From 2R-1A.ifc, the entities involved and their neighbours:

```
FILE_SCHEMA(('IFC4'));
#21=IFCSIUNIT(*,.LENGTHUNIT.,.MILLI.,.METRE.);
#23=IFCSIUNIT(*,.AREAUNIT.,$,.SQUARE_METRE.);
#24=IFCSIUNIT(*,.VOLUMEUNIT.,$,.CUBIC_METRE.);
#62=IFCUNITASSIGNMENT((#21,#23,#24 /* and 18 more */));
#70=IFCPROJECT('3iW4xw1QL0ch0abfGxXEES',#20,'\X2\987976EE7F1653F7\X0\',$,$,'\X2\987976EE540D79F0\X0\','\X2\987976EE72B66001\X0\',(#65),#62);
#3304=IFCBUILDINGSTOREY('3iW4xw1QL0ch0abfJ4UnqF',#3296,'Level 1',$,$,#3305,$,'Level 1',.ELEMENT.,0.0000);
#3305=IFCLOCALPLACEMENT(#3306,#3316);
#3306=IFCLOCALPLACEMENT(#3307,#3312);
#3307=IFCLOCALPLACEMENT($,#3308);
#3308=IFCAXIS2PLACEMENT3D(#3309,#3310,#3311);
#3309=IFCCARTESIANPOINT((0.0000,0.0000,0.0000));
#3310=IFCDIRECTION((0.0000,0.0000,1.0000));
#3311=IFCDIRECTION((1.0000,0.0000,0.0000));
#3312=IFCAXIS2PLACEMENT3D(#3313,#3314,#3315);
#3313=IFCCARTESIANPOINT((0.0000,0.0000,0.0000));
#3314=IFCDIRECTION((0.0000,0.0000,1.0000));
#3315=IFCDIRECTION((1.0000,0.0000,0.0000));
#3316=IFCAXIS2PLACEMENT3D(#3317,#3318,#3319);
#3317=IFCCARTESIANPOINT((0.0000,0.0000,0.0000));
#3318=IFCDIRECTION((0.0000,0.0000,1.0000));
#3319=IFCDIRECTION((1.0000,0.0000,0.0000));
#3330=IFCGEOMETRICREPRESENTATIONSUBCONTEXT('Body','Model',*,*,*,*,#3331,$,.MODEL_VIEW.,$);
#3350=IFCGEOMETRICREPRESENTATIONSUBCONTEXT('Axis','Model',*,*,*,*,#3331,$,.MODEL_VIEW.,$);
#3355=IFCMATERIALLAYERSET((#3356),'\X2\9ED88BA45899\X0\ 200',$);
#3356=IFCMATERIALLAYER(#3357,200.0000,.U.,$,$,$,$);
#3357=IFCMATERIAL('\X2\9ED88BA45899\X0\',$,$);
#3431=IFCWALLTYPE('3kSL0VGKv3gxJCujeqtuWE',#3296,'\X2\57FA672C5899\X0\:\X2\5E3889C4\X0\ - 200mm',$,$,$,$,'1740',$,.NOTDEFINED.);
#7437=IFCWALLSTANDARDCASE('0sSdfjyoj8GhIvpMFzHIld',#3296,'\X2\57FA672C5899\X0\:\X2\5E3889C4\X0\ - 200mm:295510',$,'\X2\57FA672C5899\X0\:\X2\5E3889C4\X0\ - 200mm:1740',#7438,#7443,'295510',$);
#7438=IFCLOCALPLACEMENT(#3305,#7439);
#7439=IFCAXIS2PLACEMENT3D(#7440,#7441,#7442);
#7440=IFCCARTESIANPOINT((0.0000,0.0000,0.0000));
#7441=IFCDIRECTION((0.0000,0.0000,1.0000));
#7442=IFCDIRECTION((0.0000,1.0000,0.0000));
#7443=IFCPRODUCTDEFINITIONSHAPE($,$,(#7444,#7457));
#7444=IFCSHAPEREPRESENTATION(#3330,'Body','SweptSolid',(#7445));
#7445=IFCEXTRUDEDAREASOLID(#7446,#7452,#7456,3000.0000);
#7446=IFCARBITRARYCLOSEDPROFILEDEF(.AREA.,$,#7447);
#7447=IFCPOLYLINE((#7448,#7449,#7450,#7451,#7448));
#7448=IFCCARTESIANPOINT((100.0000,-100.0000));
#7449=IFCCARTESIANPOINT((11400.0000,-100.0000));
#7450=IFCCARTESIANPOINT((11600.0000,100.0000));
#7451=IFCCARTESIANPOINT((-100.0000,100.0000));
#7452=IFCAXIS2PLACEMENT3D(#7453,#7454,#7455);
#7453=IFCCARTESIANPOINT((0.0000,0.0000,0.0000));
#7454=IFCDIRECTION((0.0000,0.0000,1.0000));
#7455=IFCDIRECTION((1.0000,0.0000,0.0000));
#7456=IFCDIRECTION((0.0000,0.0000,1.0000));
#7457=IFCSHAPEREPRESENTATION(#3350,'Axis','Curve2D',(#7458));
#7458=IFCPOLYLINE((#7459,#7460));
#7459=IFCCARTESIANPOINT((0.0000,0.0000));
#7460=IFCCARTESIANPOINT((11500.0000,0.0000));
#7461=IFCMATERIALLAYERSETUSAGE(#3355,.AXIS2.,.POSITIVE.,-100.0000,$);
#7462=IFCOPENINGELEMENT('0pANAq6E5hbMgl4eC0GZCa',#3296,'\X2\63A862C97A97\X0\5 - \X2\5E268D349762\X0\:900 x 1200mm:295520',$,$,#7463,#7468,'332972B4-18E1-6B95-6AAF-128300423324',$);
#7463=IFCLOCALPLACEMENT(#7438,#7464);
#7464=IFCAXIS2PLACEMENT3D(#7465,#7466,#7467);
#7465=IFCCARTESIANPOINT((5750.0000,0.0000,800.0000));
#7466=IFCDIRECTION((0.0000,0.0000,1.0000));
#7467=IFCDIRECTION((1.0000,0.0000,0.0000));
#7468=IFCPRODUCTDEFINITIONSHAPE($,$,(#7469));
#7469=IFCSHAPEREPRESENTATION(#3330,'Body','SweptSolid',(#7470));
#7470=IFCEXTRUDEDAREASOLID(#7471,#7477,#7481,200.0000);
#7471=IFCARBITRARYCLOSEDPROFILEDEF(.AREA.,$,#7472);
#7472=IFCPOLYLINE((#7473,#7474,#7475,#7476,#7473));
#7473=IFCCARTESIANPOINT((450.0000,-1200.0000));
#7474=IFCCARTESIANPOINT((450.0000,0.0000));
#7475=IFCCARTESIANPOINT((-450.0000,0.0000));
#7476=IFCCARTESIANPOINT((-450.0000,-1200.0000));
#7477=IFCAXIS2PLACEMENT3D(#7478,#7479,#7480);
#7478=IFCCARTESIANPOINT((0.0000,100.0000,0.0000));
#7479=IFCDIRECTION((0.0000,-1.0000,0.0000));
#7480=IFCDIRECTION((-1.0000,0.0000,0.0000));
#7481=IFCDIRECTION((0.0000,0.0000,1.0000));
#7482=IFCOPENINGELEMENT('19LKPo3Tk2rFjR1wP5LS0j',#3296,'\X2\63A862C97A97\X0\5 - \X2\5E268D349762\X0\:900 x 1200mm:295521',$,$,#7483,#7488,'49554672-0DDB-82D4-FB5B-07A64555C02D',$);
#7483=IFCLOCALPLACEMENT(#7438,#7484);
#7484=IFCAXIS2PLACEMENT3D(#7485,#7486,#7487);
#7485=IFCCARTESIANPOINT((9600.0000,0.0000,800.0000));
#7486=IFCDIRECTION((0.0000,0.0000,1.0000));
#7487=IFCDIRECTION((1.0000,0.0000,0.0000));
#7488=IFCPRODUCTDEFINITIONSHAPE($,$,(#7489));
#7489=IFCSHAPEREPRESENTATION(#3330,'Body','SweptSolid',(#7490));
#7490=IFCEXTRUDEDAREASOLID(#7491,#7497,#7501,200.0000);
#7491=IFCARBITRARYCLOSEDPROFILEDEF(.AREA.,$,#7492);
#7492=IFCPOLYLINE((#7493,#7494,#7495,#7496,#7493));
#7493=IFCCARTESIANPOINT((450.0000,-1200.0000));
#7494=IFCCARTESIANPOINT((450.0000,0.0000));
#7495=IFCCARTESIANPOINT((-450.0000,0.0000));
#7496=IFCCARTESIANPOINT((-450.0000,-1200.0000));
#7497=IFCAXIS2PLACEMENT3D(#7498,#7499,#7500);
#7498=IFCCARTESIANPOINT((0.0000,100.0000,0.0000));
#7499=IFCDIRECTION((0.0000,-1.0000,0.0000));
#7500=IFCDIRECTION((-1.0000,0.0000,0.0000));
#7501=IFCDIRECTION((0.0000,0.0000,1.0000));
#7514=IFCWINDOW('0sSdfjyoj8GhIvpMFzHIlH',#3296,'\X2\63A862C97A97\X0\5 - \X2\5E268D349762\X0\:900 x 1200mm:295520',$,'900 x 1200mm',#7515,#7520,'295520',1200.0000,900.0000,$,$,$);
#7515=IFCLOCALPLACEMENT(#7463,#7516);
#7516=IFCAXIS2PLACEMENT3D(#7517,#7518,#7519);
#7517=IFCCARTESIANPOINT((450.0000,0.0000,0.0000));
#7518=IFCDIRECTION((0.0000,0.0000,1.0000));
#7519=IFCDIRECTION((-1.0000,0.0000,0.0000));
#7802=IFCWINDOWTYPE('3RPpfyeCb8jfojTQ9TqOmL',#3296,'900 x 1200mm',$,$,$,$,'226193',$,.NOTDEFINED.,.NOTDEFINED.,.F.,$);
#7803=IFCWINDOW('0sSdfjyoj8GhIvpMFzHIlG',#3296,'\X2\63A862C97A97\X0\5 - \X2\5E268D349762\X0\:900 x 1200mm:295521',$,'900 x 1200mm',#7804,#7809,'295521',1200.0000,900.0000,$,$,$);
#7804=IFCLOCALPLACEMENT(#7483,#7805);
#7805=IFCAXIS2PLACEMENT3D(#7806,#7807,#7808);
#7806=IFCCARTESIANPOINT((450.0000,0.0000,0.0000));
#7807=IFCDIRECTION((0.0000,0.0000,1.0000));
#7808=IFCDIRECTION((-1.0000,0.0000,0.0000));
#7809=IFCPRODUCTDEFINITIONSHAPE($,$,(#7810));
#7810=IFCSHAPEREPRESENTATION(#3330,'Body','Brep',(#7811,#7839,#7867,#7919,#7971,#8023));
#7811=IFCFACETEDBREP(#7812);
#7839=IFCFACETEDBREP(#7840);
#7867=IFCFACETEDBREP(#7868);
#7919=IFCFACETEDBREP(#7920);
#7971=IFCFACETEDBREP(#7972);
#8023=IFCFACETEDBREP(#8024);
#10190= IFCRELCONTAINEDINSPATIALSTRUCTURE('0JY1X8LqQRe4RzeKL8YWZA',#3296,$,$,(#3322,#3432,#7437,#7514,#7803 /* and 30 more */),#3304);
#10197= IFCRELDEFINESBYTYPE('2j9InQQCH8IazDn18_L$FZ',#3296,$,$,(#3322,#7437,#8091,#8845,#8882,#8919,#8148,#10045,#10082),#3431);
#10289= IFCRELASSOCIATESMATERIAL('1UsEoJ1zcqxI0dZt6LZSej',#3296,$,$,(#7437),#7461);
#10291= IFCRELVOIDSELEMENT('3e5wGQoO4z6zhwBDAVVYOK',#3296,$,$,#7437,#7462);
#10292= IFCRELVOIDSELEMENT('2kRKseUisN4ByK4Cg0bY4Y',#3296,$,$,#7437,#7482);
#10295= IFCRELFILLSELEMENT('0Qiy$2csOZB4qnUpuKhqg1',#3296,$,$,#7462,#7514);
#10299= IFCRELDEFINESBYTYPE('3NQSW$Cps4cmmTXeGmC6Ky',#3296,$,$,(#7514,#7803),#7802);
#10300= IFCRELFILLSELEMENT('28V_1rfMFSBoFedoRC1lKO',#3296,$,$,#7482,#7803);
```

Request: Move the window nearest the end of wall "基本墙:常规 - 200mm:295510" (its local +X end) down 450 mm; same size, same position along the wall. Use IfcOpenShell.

```python
import numpy as np
import ifcopenshell
import ifcopenshell.api.geometry
import ifcopenshell.util.placement
import ifcopenshell.util.unit

model = ifcopenshell.open("2R-1A.ifc")
unit_scale = ifcopenshell.util.unit.calculate_unit_scale(model)

window = model.by_id(7803)
opening = window.FillsVoids[0].RelatingOpeningElement
dz = -0.45 / unit_scale

shift = np.array([0.0, 0.0, dz])
# The window is placed relative to its opening, so it follows when the opening moves.
matrix = ifcopenshell.util.placement.get_local_placement(opening.ObjectPlacement)
matrix[:3, 3] += shift
ifcopenshell.api.geometry.edit_object_placement(
    model, product=opening, matrix=matrix, is_si=False, should_transform_children=True
)

print(f"moved by {dz * unit_scale:+.3f} m")

model.write("2R-1A-out.ifc")
```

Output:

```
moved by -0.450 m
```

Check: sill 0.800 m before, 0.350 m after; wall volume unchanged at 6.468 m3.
